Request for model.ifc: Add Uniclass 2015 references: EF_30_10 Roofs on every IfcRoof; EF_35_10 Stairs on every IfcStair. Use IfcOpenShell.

First a look at what the model holds.

```python
import ifcopenshell

model = ifcopenshell.open("model.ifc")
print(model.schema)
print("classifications:", [c.Name for c in model.by_type("IfcClassification")])
for ifc_class in ("IfcDoor", "IfcRoof", "IfcStair", "IfcWall", "IfcWindow"):
    print(ifc_class, len(model.by_type(ifc_class)))
```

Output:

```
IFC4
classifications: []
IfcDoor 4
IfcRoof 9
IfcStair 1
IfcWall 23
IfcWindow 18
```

```python
import ifcopenshell
import ifcopenshell.api.classification

model = ifcopenshell.open("model.ifc")

system = ifcopenshell.api.classification.add_classification(model, classification="Uniclass 2015")

codes = {
    "IfcRoof": ("EF_30_10", "Roofs"),
    "IfcStair": ("EF_35_10", "Stairs"),
}
for ifc_class, (code, name) in codes.items():
    products = model.by_type(ifc_class)
    ifcopenshell.api.classification.add_reference(
        model, products=products, classification=system, identification=code, name=name
    )
    print(code, len(products))

model.write("model_rev.ifc")
```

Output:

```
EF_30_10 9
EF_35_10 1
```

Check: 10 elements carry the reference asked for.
